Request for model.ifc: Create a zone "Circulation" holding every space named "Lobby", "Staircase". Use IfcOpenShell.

First a look at what the model holds.

```python
import ifcopenshell

model = ifcopenshell.open("model.ifc")
print(model.schema)
seen = {}
for space in model.by_type("IfcSpace"):
    seen[space.LongName] = seen.get(space.LongName, 0) + 1
for name, count in sorted(seen.items(), key=str):
    print(count, "x", name)
print("zones:", [z.Name for z in model.by_type("IfcZone")][:20])
```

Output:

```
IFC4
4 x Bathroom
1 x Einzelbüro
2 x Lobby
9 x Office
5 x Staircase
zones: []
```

```python
import ifcopenshell
import ifcopenshell.api.group
import ifcopenshell.api.root

model = ifcopenshell.open("model.ifc")

names = {"Lobby", "Staircase"}
spaces = [s for s in model.by_type("IfcSpace") if s.LongName in names]

zone = ifcopenshell.api.root.create_entity(model, ifc_class="IfcZone", name="Circulation")
ifcopenshell.api.group.assign_group(model, products=spaces, group=zone)
print(len(spaces), "spaces in", zone.Name)

model.write("model_edited.ifc")
```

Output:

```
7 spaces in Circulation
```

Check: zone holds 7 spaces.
